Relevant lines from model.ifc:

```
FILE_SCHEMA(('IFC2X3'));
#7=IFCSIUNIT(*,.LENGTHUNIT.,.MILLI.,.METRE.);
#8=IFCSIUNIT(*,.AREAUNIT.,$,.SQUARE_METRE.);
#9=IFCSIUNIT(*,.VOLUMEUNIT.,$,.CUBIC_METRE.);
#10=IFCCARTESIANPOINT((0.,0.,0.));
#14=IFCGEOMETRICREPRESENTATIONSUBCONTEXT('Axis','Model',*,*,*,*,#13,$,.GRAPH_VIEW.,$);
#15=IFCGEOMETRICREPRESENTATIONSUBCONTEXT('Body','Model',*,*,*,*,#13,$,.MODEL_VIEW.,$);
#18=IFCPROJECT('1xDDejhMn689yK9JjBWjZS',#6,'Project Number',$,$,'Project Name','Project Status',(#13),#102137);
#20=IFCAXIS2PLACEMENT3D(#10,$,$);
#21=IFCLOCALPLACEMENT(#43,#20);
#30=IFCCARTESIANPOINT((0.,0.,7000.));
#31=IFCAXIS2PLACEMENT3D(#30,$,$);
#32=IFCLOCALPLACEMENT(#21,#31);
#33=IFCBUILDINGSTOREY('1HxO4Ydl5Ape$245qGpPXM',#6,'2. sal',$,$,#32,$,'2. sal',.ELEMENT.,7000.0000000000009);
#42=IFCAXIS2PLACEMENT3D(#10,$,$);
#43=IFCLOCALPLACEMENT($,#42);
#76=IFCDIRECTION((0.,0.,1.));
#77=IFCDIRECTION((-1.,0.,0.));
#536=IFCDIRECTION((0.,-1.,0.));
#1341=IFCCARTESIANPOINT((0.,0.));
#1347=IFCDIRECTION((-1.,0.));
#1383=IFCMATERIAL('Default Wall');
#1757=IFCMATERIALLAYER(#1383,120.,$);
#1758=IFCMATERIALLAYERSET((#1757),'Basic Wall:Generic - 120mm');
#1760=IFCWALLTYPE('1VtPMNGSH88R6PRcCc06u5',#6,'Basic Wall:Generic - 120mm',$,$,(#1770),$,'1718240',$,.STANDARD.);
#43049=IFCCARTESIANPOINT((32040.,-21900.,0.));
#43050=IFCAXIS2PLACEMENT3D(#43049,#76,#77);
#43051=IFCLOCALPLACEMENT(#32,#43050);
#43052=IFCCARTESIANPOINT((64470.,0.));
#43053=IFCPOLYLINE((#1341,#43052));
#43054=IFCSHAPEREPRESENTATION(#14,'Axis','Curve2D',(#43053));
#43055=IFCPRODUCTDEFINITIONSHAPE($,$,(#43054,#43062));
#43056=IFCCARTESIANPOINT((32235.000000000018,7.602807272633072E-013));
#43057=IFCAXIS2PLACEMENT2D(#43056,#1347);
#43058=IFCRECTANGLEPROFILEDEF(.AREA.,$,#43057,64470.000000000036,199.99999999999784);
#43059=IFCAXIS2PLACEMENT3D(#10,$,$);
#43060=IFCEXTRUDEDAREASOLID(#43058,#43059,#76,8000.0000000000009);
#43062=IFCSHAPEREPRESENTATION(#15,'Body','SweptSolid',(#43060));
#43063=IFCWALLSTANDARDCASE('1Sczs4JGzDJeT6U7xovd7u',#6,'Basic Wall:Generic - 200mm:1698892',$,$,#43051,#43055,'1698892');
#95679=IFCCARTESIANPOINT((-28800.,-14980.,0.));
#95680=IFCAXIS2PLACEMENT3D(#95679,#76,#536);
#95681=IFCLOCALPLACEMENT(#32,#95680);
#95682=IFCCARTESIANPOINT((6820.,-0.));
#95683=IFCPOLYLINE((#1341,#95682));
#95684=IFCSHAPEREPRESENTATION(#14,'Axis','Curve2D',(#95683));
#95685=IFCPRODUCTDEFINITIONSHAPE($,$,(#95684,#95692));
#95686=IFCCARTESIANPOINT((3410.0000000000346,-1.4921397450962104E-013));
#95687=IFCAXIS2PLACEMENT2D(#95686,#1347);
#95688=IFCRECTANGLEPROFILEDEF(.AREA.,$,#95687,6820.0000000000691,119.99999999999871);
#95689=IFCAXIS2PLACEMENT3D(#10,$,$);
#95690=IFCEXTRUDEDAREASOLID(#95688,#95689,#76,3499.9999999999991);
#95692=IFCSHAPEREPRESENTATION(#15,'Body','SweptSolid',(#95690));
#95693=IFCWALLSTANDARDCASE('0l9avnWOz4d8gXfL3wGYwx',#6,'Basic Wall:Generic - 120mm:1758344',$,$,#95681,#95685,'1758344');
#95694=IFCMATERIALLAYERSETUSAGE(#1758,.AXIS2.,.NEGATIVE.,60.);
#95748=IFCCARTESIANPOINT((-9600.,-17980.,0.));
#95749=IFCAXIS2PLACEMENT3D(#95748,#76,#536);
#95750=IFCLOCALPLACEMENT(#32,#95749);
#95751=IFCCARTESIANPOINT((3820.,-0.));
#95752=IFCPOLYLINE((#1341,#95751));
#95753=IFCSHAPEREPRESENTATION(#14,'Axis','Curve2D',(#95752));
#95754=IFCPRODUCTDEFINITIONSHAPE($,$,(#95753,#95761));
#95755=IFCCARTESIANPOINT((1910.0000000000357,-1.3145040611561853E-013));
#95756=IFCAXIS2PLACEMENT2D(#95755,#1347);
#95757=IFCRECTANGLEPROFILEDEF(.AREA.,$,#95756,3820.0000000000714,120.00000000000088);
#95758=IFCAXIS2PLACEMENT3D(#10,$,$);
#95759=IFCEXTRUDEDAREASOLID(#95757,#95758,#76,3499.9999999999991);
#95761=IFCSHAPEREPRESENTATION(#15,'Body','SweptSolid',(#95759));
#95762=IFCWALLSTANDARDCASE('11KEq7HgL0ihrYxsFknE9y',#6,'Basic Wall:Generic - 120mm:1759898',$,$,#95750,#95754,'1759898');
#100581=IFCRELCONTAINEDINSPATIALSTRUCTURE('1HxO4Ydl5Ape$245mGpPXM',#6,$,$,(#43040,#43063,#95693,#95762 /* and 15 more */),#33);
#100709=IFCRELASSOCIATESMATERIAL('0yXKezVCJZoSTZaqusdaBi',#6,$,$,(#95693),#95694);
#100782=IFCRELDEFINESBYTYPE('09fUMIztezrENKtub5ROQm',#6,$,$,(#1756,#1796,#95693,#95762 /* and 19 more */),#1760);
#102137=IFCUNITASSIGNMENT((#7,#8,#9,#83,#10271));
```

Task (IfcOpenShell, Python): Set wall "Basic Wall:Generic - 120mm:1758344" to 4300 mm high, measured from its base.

```python
import ifcopenshell
import ifcopenshell.geom
import ifcopenshell.util.representation
import ifcopenshell.util.shape

model = ifcopenshell.open("model.ifc")
settings = ifcopenshell.geom.settings()


def volume(element):
    """Net volume in cubic metres, openings subtracted."""
    shape = ifcopenshell.geom.create_shape(settings, element)
    return ifcopenshell.util.shape.get_volume(shape.geometry)


wall = model.by_guid("0l9avnWOz4d8gXfL3wGYwx")
before = volume(wall)

body = ifcopenshell.util.representation.get_representation(wall, "Model", "Body")
solid = body.Items[0]
old_height = solid.Depth
solid.Depth = 4300.0
after = volume(wall)

print(f"height {old_height:g} -> {solid.Depth:g}, volume {before:.3f} -> {after:.3f} m3")

model.write("model_edited.ifc")
```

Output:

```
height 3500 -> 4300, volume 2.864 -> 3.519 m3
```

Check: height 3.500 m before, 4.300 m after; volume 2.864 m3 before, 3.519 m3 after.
